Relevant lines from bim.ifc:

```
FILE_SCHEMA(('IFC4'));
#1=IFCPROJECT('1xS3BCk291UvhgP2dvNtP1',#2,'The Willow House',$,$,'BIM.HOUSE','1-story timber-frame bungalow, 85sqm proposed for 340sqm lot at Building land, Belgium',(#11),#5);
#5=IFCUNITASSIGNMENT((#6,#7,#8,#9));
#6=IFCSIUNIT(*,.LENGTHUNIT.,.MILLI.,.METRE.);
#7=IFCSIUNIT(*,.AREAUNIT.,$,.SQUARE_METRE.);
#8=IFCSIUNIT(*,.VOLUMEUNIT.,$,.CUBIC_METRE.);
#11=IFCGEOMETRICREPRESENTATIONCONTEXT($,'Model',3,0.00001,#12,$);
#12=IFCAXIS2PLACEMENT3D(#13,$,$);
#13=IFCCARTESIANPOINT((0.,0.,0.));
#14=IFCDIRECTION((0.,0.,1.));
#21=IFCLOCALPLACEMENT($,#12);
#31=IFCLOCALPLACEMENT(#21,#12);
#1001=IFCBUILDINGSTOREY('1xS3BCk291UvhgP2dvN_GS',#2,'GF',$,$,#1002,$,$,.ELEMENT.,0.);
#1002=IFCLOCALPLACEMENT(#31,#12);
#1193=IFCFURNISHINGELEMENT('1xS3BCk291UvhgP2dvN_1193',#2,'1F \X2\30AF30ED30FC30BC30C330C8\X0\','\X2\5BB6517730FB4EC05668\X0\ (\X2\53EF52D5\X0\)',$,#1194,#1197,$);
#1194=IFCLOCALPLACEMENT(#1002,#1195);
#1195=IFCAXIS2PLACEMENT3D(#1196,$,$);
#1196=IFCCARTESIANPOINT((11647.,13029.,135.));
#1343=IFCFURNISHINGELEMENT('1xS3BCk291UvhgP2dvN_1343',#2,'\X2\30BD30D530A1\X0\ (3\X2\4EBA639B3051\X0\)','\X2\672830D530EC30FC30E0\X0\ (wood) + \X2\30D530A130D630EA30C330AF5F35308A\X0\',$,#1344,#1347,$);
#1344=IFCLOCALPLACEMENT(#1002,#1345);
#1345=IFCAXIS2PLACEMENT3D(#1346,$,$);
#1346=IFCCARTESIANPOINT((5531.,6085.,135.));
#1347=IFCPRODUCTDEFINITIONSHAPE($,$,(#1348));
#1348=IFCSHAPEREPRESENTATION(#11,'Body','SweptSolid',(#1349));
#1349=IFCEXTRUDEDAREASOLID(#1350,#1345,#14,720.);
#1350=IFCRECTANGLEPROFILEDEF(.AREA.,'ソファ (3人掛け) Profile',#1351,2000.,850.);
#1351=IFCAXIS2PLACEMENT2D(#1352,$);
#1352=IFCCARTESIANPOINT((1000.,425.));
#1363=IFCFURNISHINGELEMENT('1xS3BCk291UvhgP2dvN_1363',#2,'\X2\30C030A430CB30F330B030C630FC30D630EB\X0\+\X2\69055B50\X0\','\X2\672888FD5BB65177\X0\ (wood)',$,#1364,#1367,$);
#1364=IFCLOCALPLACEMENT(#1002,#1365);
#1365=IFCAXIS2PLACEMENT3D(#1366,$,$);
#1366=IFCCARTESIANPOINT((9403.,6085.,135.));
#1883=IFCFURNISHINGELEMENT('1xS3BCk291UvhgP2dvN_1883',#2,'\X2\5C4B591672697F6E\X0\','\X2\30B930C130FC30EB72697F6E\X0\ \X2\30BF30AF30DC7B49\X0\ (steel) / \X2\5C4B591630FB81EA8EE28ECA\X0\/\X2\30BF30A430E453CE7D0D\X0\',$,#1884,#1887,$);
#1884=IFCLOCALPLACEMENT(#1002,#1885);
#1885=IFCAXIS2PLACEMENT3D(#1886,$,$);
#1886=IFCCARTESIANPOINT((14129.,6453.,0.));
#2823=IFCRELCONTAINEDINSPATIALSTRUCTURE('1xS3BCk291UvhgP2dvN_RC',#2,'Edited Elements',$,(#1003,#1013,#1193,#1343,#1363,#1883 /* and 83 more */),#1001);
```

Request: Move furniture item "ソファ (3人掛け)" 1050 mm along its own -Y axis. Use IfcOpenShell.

```python
import ifcopenshell
import ifcopenshell.api.geometry
import ifcopenshell.util.placement
import ifcopenshell.util.unit

model = ifcopenshell.open("bim.ifc")
unit_scale = ifcopenshell.util.unit.calculate_unit_scale(model)

item = model.by_guid("1xS3BCk291UvhgP2dvN_1343")
matrix = ifcopenshell.util.placement.get_local_placement(item.ObjectPlacement)
matrix[:3, 3] -= matrix[:3, 1] * 1.05 / unit_scale
ifcopenshell.api.geometry.edit_object_placement(model, product=item, matrix=matrix, is_si=False)

print(ifcopenshell.util.placement.get_local_placement(item.ObjectPlacement).round(3) + 0.0)

model.write("bim-out.ifc")
```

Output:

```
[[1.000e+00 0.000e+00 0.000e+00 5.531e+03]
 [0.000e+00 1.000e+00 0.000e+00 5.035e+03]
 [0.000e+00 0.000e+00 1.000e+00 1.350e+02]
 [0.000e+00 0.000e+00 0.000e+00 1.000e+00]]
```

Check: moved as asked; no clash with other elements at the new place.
